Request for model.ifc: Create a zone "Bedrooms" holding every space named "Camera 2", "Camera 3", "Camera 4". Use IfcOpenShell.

First a look at what the model holds.

```python
import ifcopenshell

model = ifcopenshell.open("model.ifc")
print(model.schema)
seen = {}
for space in model.by_type("IfcSpace"):
    seen[space.LongName] = seen.get(space.LongName, 0) + 1
for name, count in sorted(seen.items(), key=str):
    print(count, "x", name)
print("zones:", [z.Name for z in model.by_type("IfcZone")][:20])
```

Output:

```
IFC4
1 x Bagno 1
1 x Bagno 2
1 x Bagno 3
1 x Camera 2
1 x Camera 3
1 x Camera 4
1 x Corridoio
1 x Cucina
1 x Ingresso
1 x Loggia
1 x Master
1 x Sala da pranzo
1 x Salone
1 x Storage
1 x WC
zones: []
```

```python
import ifcopenshell
import ifcopenshell.api.group
import ifcopenshell.api.root

model = ifcopenshell.open("model.ifc")

names = {"Camera 2", "Camera 3", "Camera 4"}
spaces = [s for s in model.by_type("IfcSpace") if s.LongName in names]

zone = ifcopenshell.api.root.create_entity(model, ifc_class="IfcZone", name="Bedrooms")
ifcopenshell.api.group.assign_group(model, products=spaces, group=zone)
print(len(spaces), "spaces in", zone.Name)

model.write("model_v2.ifc")
```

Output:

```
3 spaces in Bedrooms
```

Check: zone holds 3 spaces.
